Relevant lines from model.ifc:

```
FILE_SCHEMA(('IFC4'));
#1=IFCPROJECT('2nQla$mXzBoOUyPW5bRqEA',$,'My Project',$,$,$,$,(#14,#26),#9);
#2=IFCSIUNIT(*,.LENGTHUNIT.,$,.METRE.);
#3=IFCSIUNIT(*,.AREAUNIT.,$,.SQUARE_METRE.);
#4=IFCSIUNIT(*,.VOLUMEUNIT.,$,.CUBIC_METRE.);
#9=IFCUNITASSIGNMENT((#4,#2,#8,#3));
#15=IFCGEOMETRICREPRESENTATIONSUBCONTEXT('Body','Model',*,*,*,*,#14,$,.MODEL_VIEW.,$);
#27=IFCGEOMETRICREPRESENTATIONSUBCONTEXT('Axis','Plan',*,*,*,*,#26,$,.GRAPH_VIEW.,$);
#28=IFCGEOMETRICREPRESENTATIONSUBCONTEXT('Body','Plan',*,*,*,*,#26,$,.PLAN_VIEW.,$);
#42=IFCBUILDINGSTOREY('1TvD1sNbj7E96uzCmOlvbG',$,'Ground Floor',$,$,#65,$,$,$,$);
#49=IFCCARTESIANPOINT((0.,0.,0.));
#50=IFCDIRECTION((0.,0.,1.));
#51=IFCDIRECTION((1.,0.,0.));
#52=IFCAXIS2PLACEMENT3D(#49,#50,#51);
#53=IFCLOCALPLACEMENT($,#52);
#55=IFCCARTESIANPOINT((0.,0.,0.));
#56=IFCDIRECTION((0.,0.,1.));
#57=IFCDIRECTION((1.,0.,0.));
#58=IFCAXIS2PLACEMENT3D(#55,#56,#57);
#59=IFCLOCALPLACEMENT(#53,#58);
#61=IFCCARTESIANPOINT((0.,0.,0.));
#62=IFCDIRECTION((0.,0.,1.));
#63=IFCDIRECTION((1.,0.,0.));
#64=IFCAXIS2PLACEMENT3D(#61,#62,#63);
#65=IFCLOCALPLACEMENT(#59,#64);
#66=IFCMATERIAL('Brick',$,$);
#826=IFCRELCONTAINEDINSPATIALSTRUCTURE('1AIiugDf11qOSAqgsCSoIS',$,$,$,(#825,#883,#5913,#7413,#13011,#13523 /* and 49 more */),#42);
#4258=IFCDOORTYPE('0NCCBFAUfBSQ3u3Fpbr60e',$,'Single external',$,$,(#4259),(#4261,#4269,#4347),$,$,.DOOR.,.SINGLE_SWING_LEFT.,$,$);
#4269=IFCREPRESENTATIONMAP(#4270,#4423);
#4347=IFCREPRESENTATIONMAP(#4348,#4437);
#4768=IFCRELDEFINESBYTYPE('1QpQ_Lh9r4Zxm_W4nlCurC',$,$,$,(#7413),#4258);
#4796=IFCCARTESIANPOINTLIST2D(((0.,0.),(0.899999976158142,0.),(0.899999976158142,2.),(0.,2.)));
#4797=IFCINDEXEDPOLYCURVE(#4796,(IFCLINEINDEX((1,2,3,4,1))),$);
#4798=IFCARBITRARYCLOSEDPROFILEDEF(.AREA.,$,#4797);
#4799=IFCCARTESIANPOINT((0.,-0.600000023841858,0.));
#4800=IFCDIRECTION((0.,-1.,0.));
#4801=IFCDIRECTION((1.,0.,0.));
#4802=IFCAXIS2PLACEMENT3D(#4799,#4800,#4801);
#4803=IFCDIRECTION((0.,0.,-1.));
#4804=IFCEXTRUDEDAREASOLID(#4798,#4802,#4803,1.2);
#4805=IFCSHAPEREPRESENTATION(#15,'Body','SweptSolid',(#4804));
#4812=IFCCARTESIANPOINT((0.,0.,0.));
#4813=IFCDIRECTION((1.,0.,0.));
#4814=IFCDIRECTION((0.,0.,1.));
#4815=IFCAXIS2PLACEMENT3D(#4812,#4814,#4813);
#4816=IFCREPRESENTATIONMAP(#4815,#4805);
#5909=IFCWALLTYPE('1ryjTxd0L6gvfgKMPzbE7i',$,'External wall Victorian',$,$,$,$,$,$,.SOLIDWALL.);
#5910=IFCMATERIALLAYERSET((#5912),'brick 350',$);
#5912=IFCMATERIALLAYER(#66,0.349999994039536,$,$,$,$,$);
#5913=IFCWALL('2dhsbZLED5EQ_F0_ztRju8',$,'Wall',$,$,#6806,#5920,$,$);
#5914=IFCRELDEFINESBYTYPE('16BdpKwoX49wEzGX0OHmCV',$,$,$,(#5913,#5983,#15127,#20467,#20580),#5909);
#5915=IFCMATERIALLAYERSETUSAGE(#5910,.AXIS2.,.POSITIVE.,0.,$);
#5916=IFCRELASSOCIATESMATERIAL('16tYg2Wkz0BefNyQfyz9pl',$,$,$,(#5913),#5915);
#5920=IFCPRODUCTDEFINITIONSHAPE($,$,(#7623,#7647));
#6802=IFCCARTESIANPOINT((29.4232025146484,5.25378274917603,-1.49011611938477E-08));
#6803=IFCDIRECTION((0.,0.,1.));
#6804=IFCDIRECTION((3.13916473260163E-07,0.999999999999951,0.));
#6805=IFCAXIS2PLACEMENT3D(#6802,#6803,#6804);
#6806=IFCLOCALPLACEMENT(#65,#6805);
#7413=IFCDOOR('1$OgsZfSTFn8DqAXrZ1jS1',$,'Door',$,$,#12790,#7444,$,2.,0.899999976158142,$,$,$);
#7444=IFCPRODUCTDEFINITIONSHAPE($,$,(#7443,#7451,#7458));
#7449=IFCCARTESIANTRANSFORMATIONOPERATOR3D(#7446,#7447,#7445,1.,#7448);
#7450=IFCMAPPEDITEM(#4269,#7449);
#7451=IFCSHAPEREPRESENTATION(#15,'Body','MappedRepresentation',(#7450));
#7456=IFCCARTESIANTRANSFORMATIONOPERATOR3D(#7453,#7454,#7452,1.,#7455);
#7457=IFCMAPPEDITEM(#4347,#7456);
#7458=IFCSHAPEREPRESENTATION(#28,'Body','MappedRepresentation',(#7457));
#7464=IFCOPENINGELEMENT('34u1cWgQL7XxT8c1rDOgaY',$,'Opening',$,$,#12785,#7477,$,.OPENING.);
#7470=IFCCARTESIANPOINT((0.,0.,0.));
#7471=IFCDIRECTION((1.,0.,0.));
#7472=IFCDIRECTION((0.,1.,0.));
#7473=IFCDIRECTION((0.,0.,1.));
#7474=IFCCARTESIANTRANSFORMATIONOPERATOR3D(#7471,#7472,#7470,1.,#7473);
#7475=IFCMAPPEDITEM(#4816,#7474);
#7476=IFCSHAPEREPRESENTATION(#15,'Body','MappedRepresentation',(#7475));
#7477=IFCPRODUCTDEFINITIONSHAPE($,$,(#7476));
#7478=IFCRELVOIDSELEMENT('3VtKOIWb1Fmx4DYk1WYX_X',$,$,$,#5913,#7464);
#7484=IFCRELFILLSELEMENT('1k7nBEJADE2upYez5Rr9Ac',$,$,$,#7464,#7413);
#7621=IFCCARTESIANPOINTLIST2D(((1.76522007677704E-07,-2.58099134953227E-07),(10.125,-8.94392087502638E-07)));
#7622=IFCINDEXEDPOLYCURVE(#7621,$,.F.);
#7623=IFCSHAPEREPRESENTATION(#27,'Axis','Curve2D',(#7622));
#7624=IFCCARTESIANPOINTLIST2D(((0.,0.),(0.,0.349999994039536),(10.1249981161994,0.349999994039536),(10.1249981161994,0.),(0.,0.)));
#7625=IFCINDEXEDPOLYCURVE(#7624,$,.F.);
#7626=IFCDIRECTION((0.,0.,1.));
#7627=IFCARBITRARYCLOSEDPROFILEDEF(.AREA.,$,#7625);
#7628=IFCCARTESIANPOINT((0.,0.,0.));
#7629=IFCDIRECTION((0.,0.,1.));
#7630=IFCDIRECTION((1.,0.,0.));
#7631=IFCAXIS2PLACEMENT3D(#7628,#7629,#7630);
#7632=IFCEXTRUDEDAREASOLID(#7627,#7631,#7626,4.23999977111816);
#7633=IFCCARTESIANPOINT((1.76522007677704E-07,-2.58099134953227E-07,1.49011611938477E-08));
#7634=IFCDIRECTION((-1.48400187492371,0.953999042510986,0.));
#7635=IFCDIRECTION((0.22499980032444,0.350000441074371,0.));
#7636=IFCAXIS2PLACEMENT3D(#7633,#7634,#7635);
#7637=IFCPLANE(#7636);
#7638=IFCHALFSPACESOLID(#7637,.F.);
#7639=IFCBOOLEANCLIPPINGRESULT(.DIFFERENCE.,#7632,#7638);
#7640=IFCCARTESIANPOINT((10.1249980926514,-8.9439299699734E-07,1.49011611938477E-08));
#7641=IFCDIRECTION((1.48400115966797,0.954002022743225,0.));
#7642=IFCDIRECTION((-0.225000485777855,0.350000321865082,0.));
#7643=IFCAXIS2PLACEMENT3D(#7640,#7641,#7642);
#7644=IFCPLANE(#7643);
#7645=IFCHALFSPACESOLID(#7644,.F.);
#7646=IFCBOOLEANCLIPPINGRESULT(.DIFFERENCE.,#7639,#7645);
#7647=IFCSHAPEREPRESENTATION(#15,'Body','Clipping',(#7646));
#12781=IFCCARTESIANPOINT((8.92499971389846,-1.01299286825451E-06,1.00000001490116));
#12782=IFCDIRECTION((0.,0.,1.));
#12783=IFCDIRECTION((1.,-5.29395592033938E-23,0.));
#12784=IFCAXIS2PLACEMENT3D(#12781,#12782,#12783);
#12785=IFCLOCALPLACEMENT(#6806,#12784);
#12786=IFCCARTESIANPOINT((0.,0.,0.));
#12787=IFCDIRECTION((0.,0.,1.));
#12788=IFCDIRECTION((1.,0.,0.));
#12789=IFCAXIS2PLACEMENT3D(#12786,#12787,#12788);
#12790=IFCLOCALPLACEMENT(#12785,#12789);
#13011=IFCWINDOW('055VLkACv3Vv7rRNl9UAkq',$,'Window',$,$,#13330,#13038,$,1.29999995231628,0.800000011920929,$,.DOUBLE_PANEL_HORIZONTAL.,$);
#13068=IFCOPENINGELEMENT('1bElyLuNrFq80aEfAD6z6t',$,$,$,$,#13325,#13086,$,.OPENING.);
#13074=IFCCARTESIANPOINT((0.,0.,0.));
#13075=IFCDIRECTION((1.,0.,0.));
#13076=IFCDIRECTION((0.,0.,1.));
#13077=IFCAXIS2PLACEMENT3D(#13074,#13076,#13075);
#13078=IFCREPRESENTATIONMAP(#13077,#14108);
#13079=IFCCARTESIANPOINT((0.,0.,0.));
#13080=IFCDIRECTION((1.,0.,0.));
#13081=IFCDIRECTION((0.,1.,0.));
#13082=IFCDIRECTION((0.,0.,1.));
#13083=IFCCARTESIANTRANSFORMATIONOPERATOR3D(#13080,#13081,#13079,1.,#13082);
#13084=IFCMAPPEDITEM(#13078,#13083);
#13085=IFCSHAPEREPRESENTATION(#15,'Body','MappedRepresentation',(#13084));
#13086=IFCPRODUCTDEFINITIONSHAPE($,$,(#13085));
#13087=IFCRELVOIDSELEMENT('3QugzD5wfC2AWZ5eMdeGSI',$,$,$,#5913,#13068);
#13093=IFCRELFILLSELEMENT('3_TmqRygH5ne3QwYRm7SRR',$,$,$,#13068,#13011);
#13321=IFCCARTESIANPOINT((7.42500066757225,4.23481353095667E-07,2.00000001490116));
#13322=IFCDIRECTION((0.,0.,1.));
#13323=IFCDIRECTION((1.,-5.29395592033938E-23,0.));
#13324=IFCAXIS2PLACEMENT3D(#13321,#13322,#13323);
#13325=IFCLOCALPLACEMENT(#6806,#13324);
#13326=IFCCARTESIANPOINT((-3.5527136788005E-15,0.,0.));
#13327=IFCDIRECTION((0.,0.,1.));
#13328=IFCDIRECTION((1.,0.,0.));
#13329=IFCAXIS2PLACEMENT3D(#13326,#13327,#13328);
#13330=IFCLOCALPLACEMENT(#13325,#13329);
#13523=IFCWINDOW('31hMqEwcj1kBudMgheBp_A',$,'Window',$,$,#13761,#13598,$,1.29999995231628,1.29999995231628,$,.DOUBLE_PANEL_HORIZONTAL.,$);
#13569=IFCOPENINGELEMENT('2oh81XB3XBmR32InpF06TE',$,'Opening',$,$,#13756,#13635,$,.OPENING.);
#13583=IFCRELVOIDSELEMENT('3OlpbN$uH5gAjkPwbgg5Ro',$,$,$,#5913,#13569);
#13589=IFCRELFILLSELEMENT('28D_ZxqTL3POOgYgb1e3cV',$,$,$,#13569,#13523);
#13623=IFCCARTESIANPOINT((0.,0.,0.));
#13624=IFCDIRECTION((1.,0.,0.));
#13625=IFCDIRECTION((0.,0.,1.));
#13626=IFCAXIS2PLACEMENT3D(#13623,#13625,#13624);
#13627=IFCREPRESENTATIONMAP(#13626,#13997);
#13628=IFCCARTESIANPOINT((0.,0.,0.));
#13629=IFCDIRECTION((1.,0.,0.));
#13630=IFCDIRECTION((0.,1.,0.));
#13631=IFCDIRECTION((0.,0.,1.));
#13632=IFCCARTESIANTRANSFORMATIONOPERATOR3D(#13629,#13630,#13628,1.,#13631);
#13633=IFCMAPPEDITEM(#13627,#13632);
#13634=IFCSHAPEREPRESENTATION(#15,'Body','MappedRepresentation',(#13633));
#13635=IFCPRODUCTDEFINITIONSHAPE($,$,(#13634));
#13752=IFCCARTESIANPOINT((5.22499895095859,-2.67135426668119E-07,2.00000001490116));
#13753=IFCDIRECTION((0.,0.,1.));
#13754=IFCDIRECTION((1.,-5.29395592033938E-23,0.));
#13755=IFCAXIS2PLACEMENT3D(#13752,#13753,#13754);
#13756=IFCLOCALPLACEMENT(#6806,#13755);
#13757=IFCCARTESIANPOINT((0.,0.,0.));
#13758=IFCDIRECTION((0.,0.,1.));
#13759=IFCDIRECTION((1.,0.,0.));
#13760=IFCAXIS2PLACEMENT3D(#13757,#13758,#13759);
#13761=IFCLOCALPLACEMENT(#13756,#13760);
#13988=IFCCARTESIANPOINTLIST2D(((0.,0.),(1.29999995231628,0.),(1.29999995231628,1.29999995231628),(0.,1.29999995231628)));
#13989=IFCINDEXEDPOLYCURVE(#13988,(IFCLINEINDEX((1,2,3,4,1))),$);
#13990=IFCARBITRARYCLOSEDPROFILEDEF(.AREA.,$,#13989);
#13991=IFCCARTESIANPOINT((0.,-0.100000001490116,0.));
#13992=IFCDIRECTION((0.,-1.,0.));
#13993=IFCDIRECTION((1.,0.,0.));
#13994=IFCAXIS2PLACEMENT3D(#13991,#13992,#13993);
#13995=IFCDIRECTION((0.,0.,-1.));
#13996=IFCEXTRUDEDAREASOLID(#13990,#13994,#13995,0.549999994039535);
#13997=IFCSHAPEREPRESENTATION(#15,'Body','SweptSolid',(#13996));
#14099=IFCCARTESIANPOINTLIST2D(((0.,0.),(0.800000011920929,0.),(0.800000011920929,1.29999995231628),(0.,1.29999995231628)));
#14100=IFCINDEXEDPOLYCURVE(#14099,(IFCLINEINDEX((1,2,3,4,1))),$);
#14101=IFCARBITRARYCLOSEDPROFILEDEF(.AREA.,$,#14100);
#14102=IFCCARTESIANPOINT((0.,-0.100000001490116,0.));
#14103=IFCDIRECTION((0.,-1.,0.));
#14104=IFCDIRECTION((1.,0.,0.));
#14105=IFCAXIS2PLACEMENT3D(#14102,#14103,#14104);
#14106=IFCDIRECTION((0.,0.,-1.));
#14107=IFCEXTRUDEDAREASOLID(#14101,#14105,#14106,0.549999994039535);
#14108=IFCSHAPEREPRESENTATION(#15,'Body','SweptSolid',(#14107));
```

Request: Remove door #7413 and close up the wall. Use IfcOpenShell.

```python
import ifcopenshell
import ifcopenshell.api.feature
import ifcopenshell.api.root
import ifcopenshell.geom
import ifcopenshell.util.shape

model = ifcopenshell.open("model.ifc")
settings = ifcopenshell.geom.settings()


def volume(element):
    """Net volume in cubic metres, openings subtracted."""
    shape = ifcopenshell.geom.create_shape(settings, element)
    return ifcopenshell.util.shape.get_volume(shape.geometry)


door = model.by_guid("1$OgsZfSTFn8DqAXrZ1jS1")
opening = door.FillsVoids[0].RelatingOpeningElement
wall = opening.VoidsElements[0].RelatingBuildingElement
before = volume(wall)

ifcopenshell.api.root.remove_product(model, product=door)
ifcopenshell.api.feature.remove_feature(model, feature=opening)

after = volume(wall)

print(f"wall volume {before:.3f} -> {after:.3f} m3")

model.write("model-out.ifc")
```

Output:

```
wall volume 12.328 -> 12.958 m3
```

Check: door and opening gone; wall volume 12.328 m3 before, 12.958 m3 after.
